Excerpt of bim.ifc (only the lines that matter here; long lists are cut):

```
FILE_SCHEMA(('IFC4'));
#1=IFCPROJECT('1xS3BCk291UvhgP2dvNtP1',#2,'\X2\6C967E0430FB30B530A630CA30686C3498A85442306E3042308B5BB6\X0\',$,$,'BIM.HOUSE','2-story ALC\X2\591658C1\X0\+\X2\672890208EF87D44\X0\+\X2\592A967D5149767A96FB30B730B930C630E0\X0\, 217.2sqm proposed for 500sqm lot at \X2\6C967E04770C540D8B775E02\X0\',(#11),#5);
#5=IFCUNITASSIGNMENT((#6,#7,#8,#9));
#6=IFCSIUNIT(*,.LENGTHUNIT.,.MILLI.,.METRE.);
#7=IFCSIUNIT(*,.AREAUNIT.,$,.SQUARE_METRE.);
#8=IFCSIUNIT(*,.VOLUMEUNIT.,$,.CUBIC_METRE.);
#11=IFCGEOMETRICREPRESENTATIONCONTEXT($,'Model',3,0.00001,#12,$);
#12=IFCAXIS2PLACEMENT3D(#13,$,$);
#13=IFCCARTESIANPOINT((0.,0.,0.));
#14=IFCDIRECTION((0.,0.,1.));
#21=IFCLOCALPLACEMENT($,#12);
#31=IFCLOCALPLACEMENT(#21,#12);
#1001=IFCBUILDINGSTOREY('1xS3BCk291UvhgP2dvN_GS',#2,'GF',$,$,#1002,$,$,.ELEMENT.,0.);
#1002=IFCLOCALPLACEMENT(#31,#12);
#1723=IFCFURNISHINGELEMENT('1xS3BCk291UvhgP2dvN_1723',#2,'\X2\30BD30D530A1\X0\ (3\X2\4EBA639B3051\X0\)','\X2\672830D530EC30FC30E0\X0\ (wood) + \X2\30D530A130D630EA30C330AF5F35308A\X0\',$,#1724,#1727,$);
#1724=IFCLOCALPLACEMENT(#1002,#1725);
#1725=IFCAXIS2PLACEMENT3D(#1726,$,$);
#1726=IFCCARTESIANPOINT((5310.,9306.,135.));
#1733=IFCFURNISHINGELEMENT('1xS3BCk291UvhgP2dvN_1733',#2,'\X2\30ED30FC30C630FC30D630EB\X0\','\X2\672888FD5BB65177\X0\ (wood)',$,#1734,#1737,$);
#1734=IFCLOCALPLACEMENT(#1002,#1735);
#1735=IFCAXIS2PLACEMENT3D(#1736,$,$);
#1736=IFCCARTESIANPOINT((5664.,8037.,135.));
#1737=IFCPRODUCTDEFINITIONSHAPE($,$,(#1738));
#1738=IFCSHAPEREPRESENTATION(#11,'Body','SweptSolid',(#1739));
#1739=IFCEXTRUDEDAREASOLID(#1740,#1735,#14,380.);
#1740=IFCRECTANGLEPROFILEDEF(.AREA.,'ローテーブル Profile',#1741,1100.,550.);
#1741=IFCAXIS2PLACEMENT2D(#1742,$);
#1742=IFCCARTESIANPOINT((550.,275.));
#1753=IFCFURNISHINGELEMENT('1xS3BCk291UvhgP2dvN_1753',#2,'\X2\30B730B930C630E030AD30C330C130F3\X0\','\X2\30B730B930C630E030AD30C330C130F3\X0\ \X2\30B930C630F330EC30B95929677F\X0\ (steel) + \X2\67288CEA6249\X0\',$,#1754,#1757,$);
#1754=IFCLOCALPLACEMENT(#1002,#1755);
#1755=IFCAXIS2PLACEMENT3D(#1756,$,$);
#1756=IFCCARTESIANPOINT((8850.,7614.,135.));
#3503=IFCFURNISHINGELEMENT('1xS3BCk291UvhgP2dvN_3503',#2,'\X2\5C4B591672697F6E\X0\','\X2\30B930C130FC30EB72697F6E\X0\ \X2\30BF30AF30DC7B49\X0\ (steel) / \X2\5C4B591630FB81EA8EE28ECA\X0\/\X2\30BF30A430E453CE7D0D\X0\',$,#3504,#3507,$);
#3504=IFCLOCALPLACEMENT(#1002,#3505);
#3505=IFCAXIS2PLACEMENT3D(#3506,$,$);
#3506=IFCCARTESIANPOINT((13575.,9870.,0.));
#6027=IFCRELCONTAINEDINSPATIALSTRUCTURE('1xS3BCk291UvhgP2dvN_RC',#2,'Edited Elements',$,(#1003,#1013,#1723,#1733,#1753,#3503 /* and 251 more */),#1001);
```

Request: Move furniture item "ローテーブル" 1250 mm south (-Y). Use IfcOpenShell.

```python
import ifcopenshell
import ifcopenshell.api.geometry
import ifcopenshell.util.placement

model = ifcopenshell.open("bim.ifc")

item = model.by_guid("1xS3BCk291UvhgP2dvN_1733")
matrix = ifcopenshell.util.placement.get_local_placement(item.ObjectPlacement)
matrix[1, 3] -= 1250.0
ifcopenshell.api.geometry.edit_object_placement(model, product=item, matrix=matrix, is_si=False)

print(ifcopenshell.util.placement.get_local_placement(item.ObjectPlacement).round(3) + 0.0)

model.write("bim_edited.ifc")
```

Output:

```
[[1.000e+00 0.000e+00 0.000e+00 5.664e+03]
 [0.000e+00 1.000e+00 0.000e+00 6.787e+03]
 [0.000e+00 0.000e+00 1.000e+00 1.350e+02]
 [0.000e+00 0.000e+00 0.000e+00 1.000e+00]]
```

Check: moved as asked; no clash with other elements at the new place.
